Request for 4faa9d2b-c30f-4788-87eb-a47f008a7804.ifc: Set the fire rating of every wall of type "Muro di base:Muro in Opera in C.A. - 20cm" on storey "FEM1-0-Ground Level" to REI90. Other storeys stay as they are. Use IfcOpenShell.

First a look at what the model holds.

```python
import ifcopenshell
import ifcopenshell.util.element

model = ifcopenshell.open("4faa9d2b-c30f-4788-87eb-a47f008a7804.ifc")
print(model.schema)
storey = next(s for s in model.by_type("IfcBuildingStorey") if s.Name == "FEM1-0-Ground Level")
walls = [e for e in ifcopenshell.util.element.get_decomposition(storey) if e.is_a("IfcWall")]
seen = {}
for e in walls:
    element_type = ifcopenshell.util.element.get_type(e)
    key = (element_type.Name if element_type != e and element_type else None, ifcopenshell.util.element.get_pset(e, "Pset_WallCommon", "FireRating"))
    seen[key] = seen.get(key, 0) + 1
for (name, value), count in sorted(seen.items(), key=str):
    print(count, "x", name, "|", value)
```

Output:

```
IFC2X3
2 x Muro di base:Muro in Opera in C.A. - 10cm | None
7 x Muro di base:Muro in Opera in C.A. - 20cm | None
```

```python
import ifcopenshell
import ifcopenshell.api.pset
import ifcopenshell.util.element

model = ifcopenshell.open("4faa9d2b-c30f-4788-87eb-a47f008a7804.ifc")

storey = next(s for s in model.by_type("IfcBuildingStorey") if s.Name == "FEM1-0-Ground Level")
walls = [e for e in ifcopenshell.util.element.get_decomposition(storey) if e.is_a("IfcWall")]

count = 0
for e in walls:
    element_type = ifcopenshell.util.element.get_type(e)
    if element_type in (None, e) or element_type.Name != "Muro di base:Muro in Opera in C.A. - 20cm":
        continue
    # add_pset returns the element's existing set when there is one.
    pset = ifcopenshell.api.pset.add_pset(model, product=e, name="Pset_WallCommon")
    ifcopenshell.api.pset.edit_pset(model, pset=pset, properties={"FireRating": "REI90"})
    count += 1

print(count, "walls updated")

model.write("4faa9d2b-c30f-4788-87eb-a47f008a7804_edited.ifc")
```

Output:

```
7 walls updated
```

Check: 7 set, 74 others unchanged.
